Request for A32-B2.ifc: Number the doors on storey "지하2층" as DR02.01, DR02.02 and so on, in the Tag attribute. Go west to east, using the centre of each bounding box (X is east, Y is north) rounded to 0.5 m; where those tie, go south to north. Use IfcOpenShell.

First a look at what the model holds.

```python
import ifcopenshell
import ifcopenshell.util.element
import ifcopenshell.util.placement

model = ifcopenshell.open("A32-B2.ifc")
print(model.schema)
storey = next(s for s in model.by_type("IfcBuildingStorey") if s.Name == "지하2층")
doors = [e for e in ifcopenshell.util.element.get_decomposition(storey) if e.is_a("IfcDoor")]
for e in sorted(doors, key=lambda e: e.id()):
    origin = ifcopenshell.util.placement.get_local_placement(e.ObjectPlacement)[:3, 3]
    print(e.id(), e.Tag, e.Name, origin.round(2) + 0.0, sep=" | ")
```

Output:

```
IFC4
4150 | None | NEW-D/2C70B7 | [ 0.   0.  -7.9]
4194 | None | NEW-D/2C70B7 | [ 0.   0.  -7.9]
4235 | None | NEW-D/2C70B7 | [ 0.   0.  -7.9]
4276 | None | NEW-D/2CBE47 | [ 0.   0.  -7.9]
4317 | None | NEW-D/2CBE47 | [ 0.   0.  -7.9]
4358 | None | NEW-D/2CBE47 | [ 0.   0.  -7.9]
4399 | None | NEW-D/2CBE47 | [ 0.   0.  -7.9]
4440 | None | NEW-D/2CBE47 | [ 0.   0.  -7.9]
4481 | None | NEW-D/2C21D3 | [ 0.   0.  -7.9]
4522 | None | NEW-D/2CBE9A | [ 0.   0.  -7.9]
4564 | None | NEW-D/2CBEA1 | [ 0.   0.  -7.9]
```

```python
import ifcopenshell
import ifcopenshell.geom
import ifcopenshell.util.element
import ifcopenshell.util.shape

model = ifcopenshell.open("A32-B2.ifc")
settings = ifcopenshell.geom.settings()
settings.set("use-world-coords", True)


def centre(element):
    shape = ifcopenshell.geom.create_shape(settings, element)
    return ifcopenshell.util.shape.get_bbox_centroid(shape.geometry)


storey = next(s for s in model.by_type("IfcBuildingStorey") if s.Name == "지하2층")
doors = [e for e in ifcopenshell.util.element.get_decomposition(storey) if e.is_a("IfcDoor")]

# Insertion points can sit at a corner or the storey origin, so sort by the geometry (in metres).
centres = {e: centre(e) for e in doors}
doors.sort(key=lambda e: (round(centres[e][0] / 0.5), centres[e][1]))

for i, e in enumerate(doors, start=1):
    number = f"DR02.{i:02d}"
    e.Tag = number
    print(e.id(), number)

model.write("A32-B2-out.ifc")
```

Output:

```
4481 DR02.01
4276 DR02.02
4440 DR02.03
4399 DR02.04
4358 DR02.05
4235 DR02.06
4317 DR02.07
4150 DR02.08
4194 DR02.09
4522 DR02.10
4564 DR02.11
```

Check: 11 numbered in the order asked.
